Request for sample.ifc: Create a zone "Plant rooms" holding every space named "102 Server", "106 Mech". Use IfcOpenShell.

First a look at what the model holds.

```python
import ifcopenshell

model = ifcopenshell.open("sample.ifc")
print(model.schema)
seen = {}
for space in model.by_type("IfcSpace"):
    seen[space.Name] = seen.get(space.Name, 0) + 1
for name, count in sorted(seen.items(), key=str):
    print(count, "x", name)
print("zones:", [z.Name for z in model.by_type("IfcZone")][:20])
```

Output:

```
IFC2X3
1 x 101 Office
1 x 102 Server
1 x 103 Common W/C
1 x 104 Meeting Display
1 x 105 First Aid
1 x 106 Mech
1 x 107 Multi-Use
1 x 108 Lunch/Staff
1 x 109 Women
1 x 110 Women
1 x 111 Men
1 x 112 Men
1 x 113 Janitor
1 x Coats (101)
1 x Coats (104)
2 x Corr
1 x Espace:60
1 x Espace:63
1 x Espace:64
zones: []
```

```python
import ifcopenshell
import ifcopenshell.api.group
import ifcopenshell.api.root

model = ifcopenshell.open("sample.ifc")

names = {"102 Server", "106 Mech"}
spaces = [s for s in model.by_type("IfcSpace") if s.Name in names]

zone = ifcopenshell.api.root.create_entity(model, ifc_class="IfcZone", name="Plant rooms")
ifcopenshell.api.group.assign_group(model, products=spaces, group=zone)
print(len(spaces), "spaces in", zone.Name)

model.write("sample_edited.ifc")
```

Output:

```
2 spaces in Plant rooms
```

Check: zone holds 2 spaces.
